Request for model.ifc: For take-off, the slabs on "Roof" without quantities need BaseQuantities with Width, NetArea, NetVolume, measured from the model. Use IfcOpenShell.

First a look at what the model holds.

```python
import ifcopenshell
import ifcopenshell.util.element
import ifcopenshell.util.unit

model = ifcopenshell.open("model.ifc")
print(model.schema)
for unit_type in ("LENGTHUNIT", "AREAUNIT", "VOLUMEUNIT"):
    print(unit_type, ifcopenshell.util.unit.calculate_unit_scale(model, unit_type))
storey = next(s for s in model.by_type("IfcBuildingStorey") if s.Name == "Roof")
slabs = [e for e in ifcopenshell.util.element.get_decomposition(storey) if e.is_a("IfcSlab")]
for e in sorted(slabs, key=lambda e: e.id()):
    print(e.id(), e.is_a(), e.Name, list(ifcopenshell.util.element.get_psets(e, qtos_only=True)), sep=" | ")
```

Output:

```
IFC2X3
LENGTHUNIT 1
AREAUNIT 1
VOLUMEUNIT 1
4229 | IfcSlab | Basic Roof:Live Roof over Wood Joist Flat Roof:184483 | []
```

```python
import ifcopenshell
import ifcopenshell.api.pset
import ifcopenshell.geom
import ifcopenshell.util.element
import ifcopenshell.util.shape
import ifcopenshell.util.unit

model = ifcopenshell.open("model.ifc")
unit_scale = ifcopenshell.util.unit.calculate_unit_scale(model)
area_scale = ifcopenshell.util.unit.calculate_unit_scale(model, "AREAUNIT")
volume_scale = ifcopenshell.util.unit.calculate_unit_scale(model, "VOLUMEUNIT")
settings = ifcopenshell.geom.settings()

storey = next(s for s in model.by_type("IfcBuildingStorey") if s.Name == "Roof")
slabs = [e for e in ifcopenshell.util.element.get_decomposition(storey) if e.is_a("IfcSlab")]

for e in sorted(slabs, key=lambda e: e.id()):
    if ifcopenshell.util.element.get_psets(e, qtos_only=True, should_inherit=False):
        continue
    # Geometry comes back in metres, in the element's own axes.
    shape = ifcopenshell.geom.create_shape(settings, e)
    values = {
        "Width": ifcopenshell.util.shape.get_z(shape.geometry) / unit_scale,
        "NetArea": ifcopenshell.util.shape.get_footprint_area(shape.geometry) / area_scale,
        "NetVolume": ifcopenshell.util.shape.get_volume(shape.geometry) / volume_scale,
    }
    qto = ifcopenshell.api.pset.add_qto(model, product=e, name="BaseQuantities")
    ifcopenshell.api.pset.edit_qto(model, qto=qto, properties=values)
    print(e.id(), {k: round(v, 3) for k, v in values.items()})

model.write("model_edited.ifc")
```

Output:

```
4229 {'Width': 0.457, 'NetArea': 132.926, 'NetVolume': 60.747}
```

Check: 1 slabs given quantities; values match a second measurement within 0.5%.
